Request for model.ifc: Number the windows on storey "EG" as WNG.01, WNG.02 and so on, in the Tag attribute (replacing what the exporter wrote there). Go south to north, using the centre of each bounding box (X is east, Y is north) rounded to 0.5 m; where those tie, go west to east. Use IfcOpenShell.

First a look at what the model holds.

```python
import ifcopenshell
import ifcopenshell.util.element
import ifcopenshell.util.placement

model = ifcopenshell.open("model.ifc")
print(model.schema)
storey = next(s for s in model.by_type("IfcBuildingStorey") if s.Name == "EG")
windows = [e for e in ifcopenshell.util.element.get_decomposition(storey) if e.is_a("IfcWindow")]
for e in sorted(windows, key=lambda e: e.id()):
    origin = ifcopenshell.util.placement.get_local_placement(e.ObjectPlacement)[:3, 3]
    print(e.id(), e.Tag, e.Name, origin.round(2) + 0.0, sep=" | ")
```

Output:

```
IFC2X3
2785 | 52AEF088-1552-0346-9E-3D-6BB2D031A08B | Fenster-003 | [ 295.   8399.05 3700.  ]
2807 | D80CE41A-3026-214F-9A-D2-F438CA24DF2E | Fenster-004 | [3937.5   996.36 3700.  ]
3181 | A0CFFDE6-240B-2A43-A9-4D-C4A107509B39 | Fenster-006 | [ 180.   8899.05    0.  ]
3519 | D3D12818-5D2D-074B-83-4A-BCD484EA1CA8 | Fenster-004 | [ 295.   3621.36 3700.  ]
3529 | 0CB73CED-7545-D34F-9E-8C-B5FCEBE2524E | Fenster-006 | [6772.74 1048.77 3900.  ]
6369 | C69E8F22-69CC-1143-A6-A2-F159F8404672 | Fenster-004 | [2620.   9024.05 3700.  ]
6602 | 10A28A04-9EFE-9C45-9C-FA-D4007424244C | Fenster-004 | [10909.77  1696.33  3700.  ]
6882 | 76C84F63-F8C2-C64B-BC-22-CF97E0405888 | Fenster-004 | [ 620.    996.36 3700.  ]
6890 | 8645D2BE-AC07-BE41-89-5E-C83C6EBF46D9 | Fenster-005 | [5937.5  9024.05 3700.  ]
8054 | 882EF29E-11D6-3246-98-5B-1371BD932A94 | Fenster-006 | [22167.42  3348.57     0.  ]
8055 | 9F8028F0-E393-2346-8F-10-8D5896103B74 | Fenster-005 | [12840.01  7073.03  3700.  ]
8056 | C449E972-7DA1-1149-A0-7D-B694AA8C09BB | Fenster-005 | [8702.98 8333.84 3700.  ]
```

```python
import ifcopenshell
import ifcopenshell.geom
import ifcopenshell.util.element
import ifcopenshell.util.shape

model = ifcopenshell.open("model.ifc")
settings = ifcopenshell.geom.settings()
settings.set("use-world-coords", True)


def centre(element):
    shape = ifcopenshell.geom.create_shape(settings, element)
    return ifcopenshell.util.shape.get_bbox_centroid(shape.geometry)


storey = next(s for s in model.by_type("IfcBuildingStorey") if s.Name == "EG")
windows = [e for e in ifcopenshell.util.element.get_decomposition(storey) if e.is_a("IfcWindow")]

# Insertion points can sit at a corner or the storey origin, so sort by the geometry (in metres).
centres = {e: centre(e) for e in windows}
windows.sort(key=lambda e: (round(centres[e][1] / 0.5), centres[e][0]))

for i, e in enumerate(windows, start=1):
    number = f"WNG.{i:02d}"
    e.Tag = number
    print(e.id(), number)

model.write("model_rev.ifc")
```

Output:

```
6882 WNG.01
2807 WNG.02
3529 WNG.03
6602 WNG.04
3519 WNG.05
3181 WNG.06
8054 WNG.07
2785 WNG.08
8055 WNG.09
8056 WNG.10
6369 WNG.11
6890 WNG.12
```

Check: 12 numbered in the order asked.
